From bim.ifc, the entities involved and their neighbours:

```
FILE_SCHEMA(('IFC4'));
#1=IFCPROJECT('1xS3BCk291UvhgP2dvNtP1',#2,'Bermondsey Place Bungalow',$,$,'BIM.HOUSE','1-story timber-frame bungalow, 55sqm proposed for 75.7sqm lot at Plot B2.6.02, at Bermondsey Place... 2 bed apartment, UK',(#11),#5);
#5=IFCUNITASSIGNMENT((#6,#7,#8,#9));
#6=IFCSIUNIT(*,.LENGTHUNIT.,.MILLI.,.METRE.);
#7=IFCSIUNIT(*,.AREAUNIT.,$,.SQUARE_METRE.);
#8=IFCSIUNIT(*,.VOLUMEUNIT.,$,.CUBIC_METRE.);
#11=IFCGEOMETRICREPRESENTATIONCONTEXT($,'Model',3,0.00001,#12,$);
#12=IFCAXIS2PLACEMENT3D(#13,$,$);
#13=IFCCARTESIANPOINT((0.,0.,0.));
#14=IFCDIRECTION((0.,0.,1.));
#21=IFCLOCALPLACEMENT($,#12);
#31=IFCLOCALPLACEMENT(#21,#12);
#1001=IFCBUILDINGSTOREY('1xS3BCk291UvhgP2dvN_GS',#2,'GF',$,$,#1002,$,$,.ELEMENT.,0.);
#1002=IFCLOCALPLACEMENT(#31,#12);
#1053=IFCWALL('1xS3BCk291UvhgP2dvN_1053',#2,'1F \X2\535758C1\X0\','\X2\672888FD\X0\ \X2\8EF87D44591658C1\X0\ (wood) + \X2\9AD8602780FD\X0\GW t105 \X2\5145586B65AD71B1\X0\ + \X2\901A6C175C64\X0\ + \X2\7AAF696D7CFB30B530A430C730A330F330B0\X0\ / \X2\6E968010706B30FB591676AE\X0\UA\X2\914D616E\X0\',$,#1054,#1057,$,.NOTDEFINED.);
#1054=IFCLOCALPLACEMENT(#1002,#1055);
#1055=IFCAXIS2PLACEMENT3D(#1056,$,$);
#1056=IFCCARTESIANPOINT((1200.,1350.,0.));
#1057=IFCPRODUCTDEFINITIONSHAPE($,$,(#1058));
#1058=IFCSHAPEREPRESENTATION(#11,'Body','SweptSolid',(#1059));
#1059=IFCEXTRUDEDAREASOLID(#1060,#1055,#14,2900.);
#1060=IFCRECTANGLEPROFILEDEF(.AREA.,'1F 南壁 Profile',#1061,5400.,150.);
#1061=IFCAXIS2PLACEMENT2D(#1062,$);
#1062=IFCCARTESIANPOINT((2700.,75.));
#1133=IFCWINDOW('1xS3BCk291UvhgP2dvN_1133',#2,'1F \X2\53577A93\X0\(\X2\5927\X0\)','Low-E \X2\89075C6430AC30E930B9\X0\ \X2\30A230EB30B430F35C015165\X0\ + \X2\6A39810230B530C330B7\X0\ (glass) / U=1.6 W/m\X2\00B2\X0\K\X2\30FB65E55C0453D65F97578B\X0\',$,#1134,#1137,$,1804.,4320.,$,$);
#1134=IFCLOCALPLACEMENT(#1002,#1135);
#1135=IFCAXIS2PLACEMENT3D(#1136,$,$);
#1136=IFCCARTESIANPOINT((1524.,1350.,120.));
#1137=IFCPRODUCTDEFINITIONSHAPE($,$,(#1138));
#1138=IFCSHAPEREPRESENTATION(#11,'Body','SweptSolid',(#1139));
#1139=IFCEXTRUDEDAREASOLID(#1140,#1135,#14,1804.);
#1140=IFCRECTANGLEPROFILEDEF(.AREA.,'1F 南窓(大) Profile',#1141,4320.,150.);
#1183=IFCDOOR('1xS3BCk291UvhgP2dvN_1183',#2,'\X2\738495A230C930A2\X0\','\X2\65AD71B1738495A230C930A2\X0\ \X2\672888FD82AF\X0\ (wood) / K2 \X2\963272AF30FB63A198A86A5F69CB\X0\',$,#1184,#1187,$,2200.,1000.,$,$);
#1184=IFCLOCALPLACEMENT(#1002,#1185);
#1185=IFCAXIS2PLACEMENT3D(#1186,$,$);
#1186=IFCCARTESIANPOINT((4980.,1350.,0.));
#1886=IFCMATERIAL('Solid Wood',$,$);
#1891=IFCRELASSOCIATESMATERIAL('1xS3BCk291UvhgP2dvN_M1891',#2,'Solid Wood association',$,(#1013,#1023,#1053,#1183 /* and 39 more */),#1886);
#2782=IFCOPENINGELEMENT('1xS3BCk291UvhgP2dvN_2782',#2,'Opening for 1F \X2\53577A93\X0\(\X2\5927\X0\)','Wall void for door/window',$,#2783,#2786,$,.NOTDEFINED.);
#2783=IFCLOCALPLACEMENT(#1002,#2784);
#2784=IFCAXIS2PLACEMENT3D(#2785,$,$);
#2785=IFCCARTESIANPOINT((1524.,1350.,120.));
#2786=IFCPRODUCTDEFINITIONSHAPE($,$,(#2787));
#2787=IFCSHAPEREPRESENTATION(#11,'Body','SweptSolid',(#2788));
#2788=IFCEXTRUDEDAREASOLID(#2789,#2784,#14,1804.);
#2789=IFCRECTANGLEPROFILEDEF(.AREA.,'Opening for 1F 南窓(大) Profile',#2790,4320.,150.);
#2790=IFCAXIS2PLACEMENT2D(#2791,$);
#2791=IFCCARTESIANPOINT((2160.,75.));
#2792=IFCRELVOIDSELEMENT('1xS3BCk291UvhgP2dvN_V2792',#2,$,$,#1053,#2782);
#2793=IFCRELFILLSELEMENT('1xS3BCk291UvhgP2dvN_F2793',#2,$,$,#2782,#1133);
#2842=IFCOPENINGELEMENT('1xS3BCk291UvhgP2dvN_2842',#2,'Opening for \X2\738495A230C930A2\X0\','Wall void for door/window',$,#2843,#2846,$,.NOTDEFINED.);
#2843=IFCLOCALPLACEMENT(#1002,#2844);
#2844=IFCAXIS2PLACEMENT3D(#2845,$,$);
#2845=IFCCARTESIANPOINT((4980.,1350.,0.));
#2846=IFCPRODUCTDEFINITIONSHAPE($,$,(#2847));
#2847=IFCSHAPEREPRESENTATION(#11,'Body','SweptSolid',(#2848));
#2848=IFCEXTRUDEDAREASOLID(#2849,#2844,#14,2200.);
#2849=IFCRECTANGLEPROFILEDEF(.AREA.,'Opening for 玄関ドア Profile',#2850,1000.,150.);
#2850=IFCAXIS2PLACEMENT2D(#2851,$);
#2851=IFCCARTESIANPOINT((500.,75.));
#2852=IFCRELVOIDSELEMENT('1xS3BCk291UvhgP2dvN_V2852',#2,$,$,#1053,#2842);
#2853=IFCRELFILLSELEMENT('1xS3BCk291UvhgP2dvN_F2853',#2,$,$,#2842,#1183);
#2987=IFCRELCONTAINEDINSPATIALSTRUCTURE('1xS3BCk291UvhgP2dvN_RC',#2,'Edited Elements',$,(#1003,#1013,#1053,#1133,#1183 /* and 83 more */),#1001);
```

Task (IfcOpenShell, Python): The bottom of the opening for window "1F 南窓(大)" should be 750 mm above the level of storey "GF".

```python
import numpy as np
import ifcopenshell
import ifcopenshell.api.geometry
import ifcopenshell.geom
import ifcopenshell.util.element
import ifcopenshell.util.placement
import ifcopenshell.util.shape
import ifcopenshell.util.unit

model = ifcopenshell.open("bim.ifc")
unit_scale = ifcopenshell.util.unit.calculate_unit_scale(model)

window = model.by_id(1133)
opening = window.FillsVoids[0].RelatingOpeningElement
storey = ifcopenshell.util.element.get_container(window, ifc_class="IfcBuildingStorey")
level = ifcopenshell.util.placement.get_local_placement(storey.ObjectPlacement)[2, 3]

# The opening's origin need not be at the sill, so measure its lowest point.
shape = ifcopenshell.geom.create_shape(ifcopenshell.geom.settings(), opening)
bottom = ifcopenshell.util.shape.get_shape_bottom_elevation(shape, shape.geometry) / unit_scale
dz = level + 750.0 - bottom

shift = np.array([0.0, 0.0, dz])
# The window is not placed relative to its opening, so move both.
for product in (opening, window):
    matrix = ifcopenshell.util.placement.get_local_placement(product.ObjectPlacement)
    matrix[:3, 3] += shift
    ifcopenshell.api.geometry.edit_object_placement(model, product=product, matrix=matrix, is_si=False)

print(f"moved by {dz * unit_scale:+.3f} m")

model.write("bim_edited.ifc")
```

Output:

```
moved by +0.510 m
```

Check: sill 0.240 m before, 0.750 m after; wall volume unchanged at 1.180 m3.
